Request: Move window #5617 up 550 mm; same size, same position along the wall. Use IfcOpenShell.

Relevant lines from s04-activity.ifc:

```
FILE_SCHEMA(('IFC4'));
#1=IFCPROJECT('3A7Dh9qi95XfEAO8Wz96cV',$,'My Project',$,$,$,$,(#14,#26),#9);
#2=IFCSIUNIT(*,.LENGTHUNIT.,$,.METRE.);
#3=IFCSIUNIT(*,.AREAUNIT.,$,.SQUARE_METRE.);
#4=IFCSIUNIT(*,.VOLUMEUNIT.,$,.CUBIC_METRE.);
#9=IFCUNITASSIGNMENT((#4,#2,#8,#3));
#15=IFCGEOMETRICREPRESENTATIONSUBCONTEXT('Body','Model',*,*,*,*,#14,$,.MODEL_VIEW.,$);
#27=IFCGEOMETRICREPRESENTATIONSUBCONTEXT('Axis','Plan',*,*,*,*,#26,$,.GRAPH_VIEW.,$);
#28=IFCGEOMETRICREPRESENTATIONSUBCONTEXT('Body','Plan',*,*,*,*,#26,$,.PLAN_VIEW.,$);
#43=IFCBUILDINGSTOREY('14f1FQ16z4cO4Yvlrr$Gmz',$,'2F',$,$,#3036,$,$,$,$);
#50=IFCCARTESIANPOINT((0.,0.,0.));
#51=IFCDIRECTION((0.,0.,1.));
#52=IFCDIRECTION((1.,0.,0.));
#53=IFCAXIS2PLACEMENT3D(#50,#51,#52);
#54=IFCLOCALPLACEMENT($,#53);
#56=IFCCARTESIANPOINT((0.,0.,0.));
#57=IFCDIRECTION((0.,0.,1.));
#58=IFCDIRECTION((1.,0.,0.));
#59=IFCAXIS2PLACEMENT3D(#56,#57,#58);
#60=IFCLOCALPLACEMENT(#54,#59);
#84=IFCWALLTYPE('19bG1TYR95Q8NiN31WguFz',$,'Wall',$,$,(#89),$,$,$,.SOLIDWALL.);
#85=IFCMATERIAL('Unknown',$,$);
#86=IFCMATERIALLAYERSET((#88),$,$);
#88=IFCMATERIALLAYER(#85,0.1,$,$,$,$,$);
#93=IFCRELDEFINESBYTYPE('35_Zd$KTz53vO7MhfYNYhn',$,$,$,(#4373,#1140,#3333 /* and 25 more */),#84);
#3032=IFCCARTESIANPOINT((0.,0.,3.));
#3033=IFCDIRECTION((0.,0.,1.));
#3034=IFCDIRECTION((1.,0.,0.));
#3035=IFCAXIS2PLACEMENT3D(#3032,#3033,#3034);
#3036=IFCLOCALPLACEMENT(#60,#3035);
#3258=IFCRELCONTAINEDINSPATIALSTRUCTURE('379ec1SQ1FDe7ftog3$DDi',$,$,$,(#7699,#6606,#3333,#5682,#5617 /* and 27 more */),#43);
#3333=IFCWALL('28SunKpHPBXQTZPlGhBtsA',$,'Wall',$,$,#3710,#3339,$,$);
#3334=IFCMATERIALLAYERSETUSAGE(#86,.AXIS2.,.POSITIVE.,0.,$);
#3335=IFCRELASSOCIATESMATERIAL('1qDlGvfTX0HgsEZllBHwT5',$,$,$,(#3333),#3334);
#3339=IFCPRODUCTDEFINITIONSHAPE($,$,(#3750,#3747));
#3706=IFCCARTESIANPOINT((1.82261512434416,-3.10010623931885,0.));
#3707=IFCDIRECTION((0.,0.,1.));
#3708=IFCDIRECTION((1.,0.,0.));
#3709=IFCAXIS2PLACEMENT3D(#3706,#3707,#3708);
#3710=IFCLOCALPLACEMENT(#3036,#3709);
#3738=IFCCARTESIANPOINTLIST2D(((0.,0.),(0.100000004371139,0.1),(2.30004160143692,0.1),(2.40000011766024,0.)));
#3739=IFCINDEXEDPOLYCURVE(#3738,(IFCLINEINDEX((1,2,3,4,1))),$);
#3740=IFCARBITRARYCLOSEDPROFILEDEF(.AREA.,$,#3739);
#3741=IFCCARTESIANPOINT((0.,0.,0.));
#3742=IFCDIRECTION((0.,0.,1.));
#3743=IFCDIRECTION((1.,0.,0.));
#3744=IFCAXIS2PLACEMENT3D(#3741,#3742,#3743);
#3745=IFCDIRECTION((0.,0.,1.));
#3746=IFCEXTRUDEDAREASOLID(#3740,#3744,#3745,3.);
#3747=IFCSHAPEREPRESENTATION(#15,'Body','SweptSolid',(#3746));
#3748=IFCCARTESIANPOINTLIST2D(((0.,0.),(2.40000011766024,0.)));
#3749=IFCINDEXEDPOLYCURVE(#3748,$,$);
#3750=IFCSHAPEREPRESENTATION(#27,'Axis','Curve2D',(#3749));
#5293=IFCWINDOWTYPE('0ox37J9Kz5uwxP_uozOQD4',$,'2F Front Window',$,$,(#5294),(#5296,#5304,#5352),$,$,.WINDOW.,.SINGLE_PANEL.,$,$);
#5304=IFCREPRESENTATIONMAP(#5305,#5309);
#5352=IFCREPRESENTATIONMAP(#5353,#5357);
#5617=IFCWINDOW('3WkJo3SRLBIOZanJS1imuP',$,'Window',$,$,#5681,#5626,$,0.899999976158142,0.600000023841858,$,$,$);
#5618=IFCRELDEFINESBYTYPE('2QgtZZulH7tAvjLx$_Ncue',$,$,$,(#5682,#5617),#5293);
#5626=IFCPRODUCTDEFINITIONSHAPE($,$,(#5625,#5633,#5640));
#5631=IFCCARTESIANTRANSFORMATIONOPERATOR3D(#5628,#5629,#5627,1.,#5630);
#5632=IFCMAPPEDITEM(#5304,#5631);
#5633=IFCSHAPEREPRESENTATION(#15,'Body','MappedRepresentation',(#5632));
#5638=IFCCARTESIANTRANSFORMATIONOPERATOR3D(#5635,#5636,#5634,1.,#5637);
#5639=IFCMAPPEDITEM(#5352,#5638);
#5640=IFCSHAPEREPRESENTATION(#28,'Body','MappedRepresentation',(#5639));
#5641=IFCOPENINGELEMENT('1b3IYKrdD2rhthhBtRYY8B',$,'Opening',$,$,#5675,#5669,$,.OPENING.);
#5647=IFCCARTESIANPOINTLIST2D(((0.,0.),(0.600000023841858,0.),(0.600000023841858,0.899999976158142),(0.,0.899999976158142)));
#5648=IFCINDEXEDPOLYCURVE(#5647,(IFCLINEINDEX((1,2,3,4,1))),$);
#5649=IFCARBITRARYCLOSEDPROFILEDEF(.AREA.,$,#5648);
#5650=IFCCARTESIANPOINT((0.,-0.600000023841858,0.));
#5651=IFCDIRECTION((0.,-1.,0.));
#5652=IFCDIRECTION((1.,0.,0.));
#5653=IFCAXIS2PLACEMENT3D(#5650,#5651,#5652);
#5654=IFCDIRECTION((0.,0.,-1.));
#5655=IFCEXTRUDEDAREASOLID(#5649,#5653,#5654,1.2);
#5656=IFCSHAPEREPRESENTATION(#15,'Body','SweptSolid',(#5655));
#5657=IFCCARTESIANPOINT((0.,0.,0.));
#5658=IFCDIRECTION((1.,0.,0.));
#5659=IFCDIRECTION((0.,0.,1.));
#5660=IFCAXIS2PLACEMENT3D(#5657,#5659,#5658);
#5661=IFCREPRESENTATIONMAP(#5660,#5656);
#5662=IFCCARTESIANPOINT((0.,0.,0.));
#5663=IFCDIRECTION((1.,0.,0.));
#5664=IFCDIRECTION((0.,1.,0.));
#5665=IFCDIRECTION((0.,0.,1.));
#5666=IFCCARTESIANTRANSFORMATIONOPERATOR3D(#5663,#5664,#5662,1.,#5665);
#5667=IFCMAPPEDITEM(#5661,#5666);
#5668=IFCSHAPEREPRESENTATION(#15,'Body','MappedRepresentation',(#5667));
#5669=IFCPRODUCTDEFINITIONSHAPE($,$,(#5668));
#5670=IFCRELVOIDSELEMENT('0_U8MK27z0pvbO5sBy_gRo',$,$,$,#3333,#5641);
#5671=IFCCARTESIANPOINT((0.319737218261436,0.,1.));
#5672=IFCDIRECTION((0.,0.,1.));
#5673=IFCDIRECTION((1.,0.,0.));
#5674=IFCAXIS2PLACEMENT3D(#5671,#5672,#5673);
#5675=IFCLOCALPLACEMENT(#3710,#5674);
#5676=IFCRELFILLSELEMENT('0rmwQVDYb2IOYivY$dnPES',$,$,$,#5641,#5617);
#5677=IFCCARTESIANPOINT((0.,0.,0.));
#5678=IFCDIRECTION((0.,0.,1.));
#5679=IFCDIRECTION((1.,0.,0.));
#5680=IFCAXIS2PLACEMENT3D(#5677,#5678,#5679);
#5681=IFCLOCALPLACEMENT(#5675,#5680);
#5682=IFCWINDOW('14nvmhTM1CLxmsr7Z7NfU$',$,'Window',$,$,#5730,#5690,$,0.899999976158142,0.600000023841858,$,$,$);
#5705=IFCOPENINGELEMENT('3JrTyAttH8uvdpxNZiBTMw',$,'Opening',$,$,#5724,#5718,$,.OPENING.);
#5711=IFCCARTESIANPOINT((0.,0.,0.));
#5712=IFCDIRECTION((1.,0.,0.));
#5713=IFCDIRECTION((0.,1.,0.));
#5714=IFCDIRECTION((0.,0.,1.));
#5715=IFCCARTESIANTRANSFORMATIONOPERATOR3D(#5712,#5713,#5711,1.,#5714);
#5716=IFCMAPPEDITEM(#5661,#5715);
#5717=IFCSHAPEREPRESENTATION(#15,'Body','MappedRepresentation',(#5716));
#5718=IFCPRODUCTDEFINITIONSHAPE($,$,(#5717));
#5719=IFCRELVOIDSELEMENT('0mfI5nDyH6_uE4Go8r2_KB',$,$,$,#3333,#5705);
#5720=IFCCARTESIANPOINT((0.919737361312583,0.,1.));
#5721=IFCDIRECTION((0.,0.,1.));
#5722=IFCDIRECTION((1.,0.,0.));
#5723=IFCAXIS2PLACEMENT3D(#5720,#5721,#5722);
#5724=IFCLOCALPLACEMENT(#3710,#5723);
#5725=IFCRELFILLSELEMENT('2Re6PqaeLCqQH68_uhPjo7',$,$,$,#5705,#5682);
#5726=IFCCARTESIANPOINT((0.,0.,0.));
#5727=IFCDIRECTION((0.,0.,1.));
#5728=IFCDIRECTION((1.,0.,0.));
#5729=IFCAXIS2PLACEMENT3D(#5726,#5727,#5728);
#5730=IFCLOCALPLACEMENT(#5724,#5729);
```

```python
import numpy as np
import ifcopenshell
import ifcopenshell.api.geometry
import ifcopenshell.util.placement
import ifcopenshell.util.unit

model = ifcopenshell.open("s04-activity.ifc")
unit_scale = ifcopenshell.util.unit.calculate_unit_scale(model)

window = model.by_id(5617)
opening = window.FillsVoids[0].RelatingOpeningElement
dz = 0.55

shift = np.array([0.0, 0.0, dz])
# The window is placed relative to its opening, so it follows when the opening moves.
matrix = ifcopenshell.util.placement.get_local_placement(opening.ObjectPlacement)
matrix[:3, 3] += shift
ifcopenshell.api.geometry.edit_object_placement(
    model, product=opening, matrix=matrix, is_si=False, should_transform_children=True
)

print(f"moved by {dz * unit_scale:+.3f} m")

model.write("s04-activity_edited.ifc")
```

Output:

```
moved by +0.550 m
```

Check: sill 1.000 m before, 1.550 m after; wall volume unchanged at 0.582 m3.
